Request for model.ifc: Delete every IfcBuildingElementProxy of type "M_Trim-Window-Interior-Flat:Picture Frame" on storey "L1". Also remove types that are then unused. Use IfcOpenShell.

First a look at what the model holds.

```python
import ifcopenshell
import ifcopenshell.util.element

model = ifcopenshell.open("model.ifc")
print(model.schema)
storey = next(s for s in model.by_type("IfcBuildingStorey") if s.Name == "L1")
proxies = [e for e in ifcopenshell.util.element.get_decomposition(storey) if e.is_a("IfcBuildingElementProxy")]
seen = {}
for e in proxies:
    element_type = ifcopenshell.util.element.get_type(e)
    name = element_type.Name if element_type not in (None, e) else None
    seen[name] = seen.get(name, 0) + 1
for name, count in sorted(seen.items(), key=str):
    print(count, "x", name)
```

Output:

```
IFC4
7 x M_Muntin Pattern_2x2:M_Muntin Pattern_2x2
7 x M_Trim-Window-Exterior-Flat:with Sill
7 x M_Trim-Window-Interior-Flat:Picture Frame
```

```python
import ifcopenshell
import ifcopenshell.api.root
import ifcopenshell.util.element

model = ifcopenshell.open("model.ifc")

storey = next(s for s in model.by_type("IfcBuildingStorey") if s.Name == "L1")
proxies = [e for e in ifcopenshell.util.element.get_decomposition(storey) if e.is_a("IfcBuildingElementProxy")]
targets = [e for e in proxies if (t := ifcopenshell.util.element.get_type(e)) not in (None, e) and t.Name == "M_Trim-Window-Interior-Flat:Picture Frame"]
types = {ifcopenshell.util.element.get_type(e) for e in targets} - {None, *targets}

for e in targets:
    ifcopenshell.api.root.remove_product(model, product=e)
print(len(targets), "removed")

unused = [t for t in types if not ifcopenshell.util.element.get_types(t)]
for t in unused:
    ifcopenshell.api.root.remove_product(model, product=t)
print(len(unused), "unused types removed")

model.write("model_v2.ifc")
```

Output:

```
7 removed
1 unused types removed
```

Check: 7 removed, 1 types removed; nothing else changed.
